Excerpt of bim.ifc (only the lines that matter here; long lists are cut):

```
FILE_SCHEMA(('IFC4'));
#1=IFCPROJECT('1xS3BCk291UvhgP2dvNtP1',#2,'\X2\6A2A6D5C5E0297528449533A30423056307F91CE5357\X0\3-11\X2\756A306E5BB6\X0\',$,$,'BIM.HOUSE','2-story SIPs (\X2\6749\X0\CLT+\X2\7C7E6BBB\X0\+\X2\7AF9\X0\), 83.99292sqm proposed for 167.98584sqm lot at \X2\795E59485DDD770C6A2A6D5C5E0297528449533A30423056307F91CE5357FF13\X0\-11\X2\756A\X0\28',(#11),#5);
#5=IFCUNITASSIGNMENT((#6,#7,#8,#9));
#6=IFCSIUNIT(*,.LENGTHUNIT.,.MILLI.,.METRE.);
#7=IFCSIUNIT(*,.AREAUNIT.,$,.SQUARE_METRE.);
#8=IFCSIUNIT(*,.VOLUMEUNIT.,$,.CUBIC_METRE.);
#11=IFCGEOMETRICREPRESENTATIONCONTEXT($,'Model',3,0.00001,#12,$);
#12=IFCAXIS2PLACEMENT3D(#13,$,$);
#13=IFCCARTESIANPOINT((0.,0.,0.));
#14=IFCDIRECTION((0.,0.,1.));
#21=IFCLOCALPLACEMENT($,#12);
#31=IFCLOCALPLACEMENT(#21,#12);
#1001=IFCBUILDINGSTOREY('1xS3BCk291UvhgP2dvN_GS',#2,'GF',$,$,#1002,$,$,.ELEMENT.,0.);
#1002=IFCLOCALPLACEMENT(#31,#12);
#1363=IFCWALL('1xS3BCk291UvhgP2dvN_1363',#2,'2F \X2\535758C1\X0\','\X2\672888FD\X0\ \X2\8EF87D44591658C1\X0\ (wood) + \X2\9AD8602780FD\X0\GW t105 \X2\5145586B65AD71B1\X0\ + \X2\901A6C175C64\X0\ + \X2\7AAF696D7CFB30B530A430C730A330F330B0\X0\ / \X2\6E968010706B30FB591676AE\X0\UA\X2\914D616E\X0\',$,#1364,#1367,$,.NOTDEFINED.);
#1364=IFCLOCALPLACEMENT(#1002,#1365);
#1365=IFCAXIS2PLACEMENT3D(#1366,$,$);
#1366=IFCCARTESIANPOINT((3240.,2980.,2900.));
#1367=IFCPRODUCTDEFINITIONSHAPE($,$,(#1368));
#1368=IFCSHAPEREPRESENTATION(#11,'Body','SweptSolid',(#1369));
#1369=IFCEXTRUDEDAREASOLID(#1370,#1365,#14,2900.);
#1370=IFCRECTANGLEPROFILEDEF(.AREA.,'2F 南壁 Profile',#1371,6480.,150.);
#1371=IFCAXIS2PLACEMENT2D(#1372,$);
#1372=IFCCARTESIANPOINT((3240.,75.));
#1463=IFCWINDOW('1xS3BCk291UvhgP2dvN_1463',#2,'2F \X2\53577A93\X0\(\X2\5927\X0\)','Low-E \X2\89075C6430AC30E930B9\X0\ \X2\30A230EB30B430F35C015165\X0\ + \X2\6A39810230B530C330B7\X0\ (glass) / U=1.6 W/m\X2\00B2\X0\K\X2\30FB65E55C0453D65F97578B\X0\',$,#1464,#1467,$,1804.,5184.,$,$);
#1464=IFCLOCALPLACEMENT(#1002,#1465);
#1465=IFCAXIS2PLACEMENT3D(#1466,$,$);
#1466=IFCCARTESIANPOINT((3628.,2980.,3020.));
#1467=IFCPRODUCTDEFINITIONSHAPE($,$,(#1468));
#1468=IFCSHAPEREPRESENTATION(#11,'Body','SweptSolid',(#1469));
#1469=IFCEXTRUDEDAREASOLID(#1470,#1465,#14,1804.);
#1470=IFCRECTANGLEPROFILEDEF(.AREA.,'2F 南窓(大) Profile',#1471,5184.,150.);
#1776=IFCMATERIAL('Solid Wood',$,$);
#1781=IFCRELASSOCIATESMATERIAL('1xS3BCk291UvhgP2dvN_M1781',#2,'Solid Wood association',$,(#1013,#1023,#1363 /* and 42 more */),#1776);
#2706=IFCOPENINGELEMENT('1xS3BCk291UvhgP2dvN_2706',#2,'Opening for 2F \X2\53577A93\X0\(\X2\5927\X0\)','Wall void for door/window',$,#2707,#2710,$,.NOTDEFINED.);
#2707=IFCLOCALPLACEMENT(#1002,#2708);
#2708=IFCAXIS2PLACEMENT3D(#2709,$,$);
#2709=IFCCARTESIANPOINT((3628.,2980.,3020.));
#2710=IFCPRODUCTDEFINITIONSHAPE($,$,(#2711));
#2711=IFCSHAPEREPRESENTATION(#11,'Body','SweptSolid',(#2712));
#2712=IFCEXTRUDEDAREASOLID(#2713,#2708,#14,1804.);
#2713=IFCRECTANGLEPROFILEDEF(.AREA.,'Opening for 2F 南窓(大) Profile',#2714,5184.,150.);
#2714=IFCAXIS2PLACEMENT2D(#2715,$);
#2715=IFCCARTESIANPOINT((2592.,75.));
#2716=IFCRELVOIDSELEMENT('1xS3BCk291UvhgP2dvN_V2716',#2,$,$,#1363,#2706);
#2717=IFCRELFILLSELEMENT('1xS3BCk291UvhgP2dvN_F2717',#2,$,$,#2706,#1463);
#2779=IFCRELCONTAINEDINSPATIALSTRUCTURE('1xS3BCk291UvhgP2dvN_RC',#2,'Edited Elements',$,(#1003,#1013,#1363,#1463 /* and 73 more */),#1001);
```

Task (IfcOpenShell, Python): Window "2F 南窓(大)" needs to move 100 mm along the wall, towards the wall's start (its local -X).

```python
import ifcopenshell
import ifcopenshell.api.geometry
import ifcopenshell.util.placement
import ifcopenshell.util.unit

model = ifcopenshell.open("bim.ifc")
unit_scale = ifcopenshell.util.unit.calculate_unit_scale(model)

window = model.by_guid("1xS3BCk291UvhgP2dvN_1463")
opening = window.FillsVoids[0].RelatingOpeningElement
wall = opening.VoidsElements[0].RelatingBuildingElement

wall_matrix = ifcopenshell.util.placement.get_local_placement(wall.ObjectPlacement)
shift = wall_matrix[:3, 0] * -0.1 / unit_scale
before = ifcopenshell.util.placement.get_local_placement(window.ObjectPlacement)[:3, 3].copy()

# The window is not placed relative to its opening, so move both.
for product in (opening, window):
    matrix = ifcopenshell.util.placement.get_local_placement(product.ObjectPlacement)
    matrix[:3, 3] += shift
    ifcopenshell.api.geometry.edit_object_placement(model, product=product, matrix=matrix, is_si=False)

after = ifcopenshell.util.placement.get_local_placement(window.ObjectPlacement)[:3, 3]
print("window moved by", (after - before).round(3) + 0.0)

model.write("bim_v2.ifc")
```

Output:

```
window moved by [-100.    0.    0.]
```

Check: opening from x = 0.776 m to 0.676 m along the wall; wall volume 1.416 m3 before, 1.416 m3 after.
